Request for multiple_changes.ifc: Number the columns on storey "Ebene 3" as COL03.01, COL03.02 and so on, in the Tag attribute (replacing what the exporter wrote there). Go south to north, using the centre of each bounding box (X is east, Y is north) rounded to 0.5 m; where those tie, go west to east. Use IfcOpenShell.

First a look at what the model holds.

```python
import ifcopenshell
import ifcopenshell.util.element
import ifcopenshell.util.placement

model = ifcopenshell.open("multiple_changes.ifc")
print(model.schema)
storey = next(s for s in model.by_type("IfcBuildingStorey") if s.Name == "Ebene 3")
columns = [e for e in ifcopenshell.util.element.get_decomposition(storey) if e.is_a("IfcColumn")]
for e in sorted(columns, key=lambda e: e.id()):
    origin = ifcopenshell.util.placement.get_local_placement(e.ObjectPlacement)[:3, 3]
    print(e.id(), e.Tag, e.Name, origin.round(2) + 0.0, sep=" | ")
```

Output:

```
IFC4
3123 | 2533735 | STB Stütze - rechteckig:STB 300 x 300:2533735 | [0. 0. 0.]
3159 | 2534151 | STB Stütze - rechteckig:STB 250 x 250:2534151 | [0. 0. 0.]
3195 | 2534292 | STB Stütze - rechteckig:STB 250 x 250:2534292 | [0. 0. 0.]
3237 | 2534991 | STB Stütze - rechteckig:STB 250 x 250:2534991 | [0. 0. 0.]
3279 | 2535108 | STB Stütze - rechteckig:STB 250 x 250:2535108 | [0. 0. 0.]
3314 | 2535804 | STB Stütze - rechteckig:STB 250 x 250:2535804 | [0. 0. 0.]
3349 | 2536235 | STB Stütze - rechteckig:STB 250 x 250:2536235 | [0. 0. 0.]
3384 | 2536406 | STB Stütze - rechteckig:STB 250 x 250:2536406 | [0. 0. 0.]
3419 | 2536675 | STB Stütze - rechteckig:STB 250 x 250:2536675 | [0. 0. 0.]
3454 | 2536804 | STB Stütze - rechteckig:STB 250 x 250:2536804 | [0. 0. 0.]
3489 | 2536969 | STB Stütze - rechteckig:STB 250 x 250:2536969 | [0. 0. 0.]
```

```python
import ifcopenshell
import ifcopenshell.geom
import ifcopenshell.util.element
import ifcopenshell.util.shape

model = ifcopenshell.open("multiple_changes.ifc")
settings = ifcopenshell.geom.settings()
settings.set("use-world-coords", True)


def centre(element):
    shape = ifcopenshell.geom.create_shape(settings, element)
    return ifcopenshell.util.shape.get_bbox_centroid(shape.geometry)


storey = next(s for s in model.by_type("IfcBuildingStorey") if s.Name == "Ebene 3")
columns = [e for e in ifcopenshell.util.element.get_decomposition(storey) if e.is_a("IfcColumn")]

# Insertion points can sit at a corner or the storey origin, so sort by the geometry (in metres).
centres = {e: centre(e) for e in columns}
columns.sort(key=lambda e: (round(centres[e][1] / 0.5), centres[e][0]))

for i, e in enumerate(columns, start=1):
    number = f"COL03.{i:02d}"
    e.Tag = number
    print(e.id(), number)

model.write("multiple_changes_updated.ifc")
```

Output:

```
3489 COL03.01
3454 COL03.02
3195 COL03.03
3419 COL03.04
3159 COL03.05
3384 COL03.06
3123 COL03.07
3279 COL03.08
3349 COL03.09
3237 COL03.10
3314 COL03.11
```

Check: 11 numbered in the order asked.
